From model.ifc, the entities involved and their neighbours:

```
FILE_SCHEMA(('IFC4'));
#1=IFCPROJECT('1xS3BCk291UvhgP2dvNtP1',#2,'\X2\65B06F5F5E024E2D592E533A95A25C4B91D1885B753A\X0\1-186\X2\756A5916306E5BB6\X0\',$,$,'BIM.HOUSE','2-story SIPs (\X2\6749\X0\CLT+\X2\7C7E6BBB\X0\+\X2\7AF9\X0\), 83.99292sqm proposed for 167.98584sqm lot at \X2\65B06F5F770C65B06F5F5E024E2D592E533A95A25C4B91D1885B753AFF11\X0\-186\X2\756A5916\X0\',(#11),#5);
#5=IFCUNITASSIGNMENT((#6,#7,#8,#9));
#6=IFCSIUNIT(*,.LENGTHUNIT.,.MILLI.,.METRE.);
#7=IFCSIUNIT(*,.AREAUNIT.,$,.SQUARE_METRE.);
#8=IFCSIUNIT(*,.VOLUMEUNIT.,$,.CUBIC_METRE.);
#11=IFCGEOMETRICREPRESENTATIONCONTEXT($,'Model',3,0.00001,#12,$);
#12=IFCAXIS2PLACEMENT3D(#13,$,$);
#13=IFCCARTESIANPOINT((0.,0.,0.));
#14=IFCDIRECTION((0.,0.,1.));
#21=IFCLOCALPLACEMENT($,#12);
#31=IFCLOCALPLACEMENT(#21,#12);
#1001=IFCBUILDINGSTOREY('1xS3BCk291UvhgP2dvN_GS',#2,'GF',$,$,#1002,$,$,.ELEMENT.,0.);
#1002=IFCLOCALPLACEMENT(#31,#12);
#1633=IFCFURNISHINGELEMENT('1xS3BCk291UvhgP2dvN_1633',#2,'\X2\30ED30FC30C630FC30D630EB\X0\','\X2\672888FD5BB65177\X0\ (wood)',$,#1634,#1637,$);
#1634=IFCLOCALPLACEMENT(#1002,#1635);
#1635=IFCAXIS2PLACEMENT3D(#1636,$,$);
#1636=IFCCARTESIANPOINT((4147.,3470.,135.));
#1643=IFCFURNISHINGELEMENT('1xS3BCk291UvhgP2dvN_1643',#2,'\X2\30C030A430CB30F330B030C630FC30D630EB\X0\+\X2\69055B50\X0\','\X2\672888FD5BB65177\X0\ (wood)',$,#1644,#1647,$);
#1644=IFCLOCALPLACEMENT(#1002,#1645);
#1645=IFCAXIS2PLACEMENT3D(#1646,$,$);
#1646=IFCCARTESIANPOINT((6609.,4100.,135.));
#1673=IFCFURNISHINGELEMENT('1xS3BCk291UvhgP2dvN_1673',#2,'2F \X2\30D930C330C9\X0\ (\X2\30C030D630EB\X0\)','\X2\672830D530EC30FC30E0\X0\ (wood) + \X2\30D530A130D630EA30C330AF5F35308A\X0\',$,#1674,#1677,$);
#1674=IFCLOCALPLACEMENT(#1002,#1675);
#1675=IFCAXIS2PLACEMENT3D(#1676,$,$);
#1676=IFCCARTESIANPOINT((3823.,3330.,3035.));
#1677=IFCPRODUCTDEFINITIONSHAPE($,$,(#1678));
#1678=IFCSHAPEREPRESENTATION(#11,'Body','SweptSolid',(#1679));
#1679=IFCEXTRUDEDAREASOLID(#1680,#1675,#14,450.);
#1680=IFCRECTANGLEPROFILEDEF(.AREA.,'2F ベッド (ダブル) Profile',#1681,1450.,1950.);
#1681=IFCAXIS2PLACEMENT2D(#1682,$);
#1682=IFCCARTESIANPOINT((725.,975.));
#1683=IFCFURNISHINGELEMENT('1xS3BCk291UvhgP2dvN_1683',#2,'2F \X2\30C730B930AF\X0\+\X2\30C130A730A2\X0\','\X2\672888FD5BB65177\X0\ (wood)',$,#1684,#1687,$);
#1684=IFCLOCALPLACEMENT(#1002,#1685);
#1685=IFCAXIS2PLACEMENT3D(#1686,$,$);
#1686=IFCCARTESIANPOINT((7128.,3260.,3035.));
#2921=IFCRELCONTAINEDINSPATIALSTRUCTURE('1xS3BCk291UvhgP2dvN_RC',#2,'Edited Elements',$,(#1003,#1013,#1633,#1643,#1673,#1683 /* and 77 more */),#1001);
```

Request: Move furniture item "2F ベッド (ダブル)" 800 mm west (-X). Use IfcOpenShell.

```python
import ifcopenshell
import ifcopenshell.api.geometry
import ifcopenshell.util.placement
import ifcopenshell.util.unit

model = ifcopenshell.open("model.ifc")
unit_scale = ifcopenshell.util.unit.calculate_unit_scale(model)

item = model.by_guid("1xS3BCk291UvhgP2dvN_1673")
matrix = ifcopenshell.util.placement.get_local_placement(item.ObjectPlacement)
matrix[0, 3] -= 0.8 / unit_scale
ifcopenshell.api.geometry.edit_object_placement(model, product=item, matrix=matrix, is_si=False)

print(ifcopenshell.util.placement.get_local_placement(item.ObjectPlacement).round(3) + 0.0)

model.write("model_edited.ifc")
```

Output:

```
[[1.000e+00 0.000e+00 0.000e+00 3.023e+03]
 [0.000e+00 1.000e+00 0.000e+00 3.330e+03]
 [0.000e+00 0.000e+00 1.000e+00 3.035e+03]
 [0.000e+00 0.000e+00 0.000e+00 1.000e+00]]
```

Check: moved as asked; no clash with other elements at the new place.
